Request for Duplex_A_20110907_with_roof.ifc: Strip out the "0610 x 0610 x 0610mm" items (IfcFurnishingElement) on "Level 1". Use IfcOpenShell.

First a look at what the model holds.

```python
import ifcopenshell
import ifcopenshell.util.element

model = ifcopenshell.open("Duplex_A_20110907_with_roof.ifc")
print(model.schema)
storey = next(s for s in model.by_type("IfcBuildingStorey") if s.Name == "Level 1")
furniture = [e for e in ifcopenshell.util.element.get_decomposition(storey) if e.is_a("IfcFurnishingElement")]
seen = {}
for e in furniture:
    element_type = ifcopenshell.util.element.get_type(e)
    name = element_type.Name if element_type not in (None, e) else None
    seen[name] = seen.get(name, 0) + 1
for name, count in sorted(seen.items(), key=str):
    print(count, "x", name)
```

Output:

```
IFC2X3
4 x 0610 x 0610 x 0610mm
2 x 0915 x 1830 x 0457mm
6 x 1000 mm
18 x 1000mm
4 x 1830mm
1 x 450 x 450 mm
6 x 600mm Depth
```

```python
import ifcopenshell
import ifcopenshell.api.root
import ifcopenshell.util.element

model = ifcopenshell.open("Duplex_A_20110907_with_roof.ifc")

storey = next(s for s in model.by_type("IfcBuildingStorey") if s.Name == "Level 1")
furniture = [e for e in ifcopenshell.util.element.get_decomposition(storey) if e.is_a("IfcFurnishingElement")]
targets = [e for e in furniture if (t := ifcopenshell.util.element.get_type(e)) not in (None, e) and t.Name == "0610 x 0610 x 0610mm"]

for e in targets:
    ifcopenshell.api.root.remove_product(model, product=e)
print(len(targets), "removed")

model.write("Duplex_A_20110907_with_roof_rev.ifc")
```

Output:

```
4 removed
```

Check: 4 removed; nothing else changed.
